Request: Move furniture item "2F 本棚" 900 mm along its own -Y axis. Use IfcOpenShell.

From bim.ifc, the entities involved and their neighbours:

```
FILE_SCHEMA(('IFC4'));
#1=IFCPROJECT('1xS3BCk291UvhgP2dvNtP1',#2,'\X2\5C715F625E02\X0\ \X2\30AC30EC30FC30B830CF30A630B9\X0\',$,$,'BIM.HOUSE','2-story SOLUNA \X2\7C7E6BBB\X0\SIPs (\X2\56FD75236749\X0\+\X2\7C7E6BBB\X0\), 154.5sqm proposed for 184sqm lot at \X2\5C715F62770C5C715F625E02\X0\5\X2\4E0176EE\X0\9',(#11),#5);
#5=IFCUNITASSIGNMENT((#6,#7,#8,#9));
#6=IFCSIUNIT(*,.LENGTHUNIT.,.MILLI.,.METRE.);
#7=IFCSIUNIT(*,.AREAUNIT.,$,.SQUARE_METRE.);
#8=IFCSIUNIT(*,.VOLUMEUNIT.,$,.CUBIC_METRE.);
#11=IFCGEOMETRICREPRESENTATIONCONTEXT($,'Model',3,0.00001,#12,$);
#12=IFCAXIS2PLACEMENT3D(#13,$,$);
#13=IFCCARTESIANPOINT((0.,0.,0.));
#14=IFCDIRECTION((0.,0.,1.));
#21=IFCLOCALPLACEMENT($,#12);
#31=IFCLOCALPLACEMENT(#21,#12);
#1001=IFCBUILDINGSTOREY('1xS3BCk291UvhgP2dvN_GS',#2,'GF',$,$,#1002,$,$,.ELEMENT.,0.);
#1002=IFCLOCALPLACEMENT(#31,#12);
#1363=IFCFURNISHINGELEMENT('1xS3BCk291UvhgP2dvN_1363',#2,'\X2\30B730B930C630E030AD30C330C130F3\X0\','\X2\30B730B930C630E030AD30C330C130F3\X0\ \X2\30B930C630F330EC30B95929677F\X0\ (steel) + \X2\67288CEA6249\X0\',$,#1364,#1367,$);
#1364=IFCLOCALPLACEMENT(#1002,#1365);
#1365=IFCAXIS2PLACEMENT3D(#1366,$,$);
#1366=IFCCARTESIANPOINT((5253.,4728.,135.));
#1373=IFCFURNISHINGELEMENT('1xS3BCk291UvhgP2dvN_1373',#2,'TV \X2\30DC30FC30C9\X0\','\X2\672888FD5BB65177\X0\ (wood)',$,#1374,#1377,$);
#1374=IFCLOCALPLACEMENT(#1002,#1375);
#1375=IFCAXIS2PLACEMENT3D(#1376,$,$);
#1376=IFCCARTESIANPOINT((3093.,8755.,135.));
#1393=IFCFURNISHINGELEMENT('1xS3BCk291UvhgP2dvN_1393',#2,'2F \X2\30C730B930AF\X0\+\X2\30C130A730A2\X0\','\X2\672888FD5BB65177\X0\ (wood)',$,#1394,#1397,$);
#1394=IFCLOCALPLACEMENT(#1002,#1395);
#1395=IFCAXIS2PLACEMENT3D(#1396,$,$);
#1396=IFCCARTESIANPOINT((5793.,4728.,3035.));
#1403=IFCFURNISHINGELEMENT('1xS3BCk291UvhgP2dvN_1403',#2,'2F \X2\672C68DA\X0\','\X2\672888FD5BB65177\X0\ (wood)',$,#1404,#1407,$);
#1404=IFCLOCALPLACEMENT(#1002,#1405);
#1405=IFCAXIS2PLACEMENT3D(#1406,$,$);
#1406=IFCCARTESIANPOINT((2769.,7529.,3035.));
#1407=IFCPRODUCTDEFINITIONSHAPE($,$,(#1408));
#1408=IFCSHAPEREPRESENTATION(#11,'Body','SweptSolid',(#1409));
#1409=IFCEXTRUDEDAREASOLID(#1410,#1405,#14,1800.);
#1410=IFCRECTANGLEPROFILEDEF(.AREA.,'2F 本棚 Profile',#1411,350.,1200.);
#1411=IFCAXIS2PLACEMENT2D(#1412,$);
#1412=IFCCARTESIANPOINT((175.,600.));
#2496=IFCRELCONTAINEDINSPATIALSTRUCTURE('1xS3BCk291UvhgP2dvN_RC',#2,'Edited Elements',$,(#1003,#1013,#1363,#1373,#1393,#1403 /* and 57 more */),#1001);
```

```python
import ifcopenshell
import ifcopenshell.api.geometry
import ifcopenshell.util.placement

model = ifcopenshell.open("bim.ifc")

item = model.by_guid("1xS3BCk291UvhgP2dvN_1403")
matrix = ifcopenshell.util.placement.get_local_placement(item.ObjectPlacement)
matrix[:3, 3] -= matrix[:3, 1] * 900.0
ifcopenshell.api.geometry.edit_object_placement(model, product=item, matrix=matrix, is_si=False)

print(ifcopenshell.util.placement.get_local_placement(item.ObjectPlacement).round(3) + 0.0)

model.write("bim_updated.ifc")
```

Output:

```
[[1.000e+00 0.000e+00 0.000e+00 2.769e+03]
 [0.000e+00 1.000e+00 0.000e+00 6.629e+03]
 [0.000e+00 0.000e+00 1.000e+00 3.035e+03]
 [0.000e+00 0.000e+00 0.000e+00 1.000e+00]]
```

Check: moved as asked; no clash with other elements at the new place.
